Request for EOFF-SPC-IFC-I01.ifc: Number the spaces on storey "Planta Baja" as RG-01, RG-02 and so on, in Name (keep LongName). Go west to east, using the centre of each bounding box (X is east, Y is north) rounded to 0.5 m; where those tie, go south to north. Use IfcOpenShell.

First a look at what the model holds.

```python
import ifcopenshell
import ifcopenshell.util.element
import ifcopenshell.util.placement

model = ifcopenshell.open("EOFF-SPC-IFC-I01.ifc")
print(model.schema)
storey = next(s for s in model.by_type("IfcBuildingStorey") if s.Name == "Planta Baja")
spaces = [e for e in ifcopenshell.util.element.get_decomposition(storey) if e.is_a("IfcSpace")]
for e in sorted(spaces, key=lambda e: e.id()):
    origin = ifcopenshell.util.placement.get_local_placement(e.ObjectPlacement)[:3, 3]
    print(e.id(), e.Name, e.LongName, origin.round(2) + 0.0, sep=" | ")
```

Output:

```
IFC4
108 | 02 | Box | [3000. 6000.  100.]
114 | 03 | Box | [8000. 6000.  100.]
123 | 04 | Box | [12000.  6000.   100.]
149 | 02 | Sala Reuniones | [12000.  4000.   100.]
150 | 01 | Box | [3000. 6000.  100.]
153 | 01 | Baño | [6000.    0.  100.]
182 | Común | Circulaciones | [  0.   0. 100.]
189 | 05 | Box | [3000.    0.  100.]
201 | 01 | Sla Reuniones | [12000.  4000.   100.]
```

```python
import ifcopenshell
import ifcopenshell.geom
import ifcopenshell.util.element
import ifcopenshell.util.shape

model = ifcopenshell.open("EOFF-SPC-IFC-I01.ifc")
settings = ifcopenshell.geom.settings()
settings.set("use-world-coords", True)


def centre(element):
    shape = ifcopenshell.geom.create_shape(settings, element)
    return ifcopenshell.util.shape.get_bbox_centroid(shape.geometry)


storey = next(s for s in model.by_type("IfcBuildingStorey") if s.Name == "Planta Baja")
spaces = [e for e in ifcopenshell.util.element.get_decomposition(storey) if e.is_a("IfcSpace")]

# Insertion points can sit at a corner or the storey origin, so sort by the geometry (in metres).
centres = {e: centre(e) for e in spaces}
spaces.sort(key=lambda e: (round(centres[e][0] / 0.5), centres[e][1]))

for i, e in enumerate(spaces, start=1):
    number = f"RG-{i:02d}"
    e.Name = number
    print(e.id(), number)

model.write("EOFF-SPC-IFC-I01_edited.ifc")
```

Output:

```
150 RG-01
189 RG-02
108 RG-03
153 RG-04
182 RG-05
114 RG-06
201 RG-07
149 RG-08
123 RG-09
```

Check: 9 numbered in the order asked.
